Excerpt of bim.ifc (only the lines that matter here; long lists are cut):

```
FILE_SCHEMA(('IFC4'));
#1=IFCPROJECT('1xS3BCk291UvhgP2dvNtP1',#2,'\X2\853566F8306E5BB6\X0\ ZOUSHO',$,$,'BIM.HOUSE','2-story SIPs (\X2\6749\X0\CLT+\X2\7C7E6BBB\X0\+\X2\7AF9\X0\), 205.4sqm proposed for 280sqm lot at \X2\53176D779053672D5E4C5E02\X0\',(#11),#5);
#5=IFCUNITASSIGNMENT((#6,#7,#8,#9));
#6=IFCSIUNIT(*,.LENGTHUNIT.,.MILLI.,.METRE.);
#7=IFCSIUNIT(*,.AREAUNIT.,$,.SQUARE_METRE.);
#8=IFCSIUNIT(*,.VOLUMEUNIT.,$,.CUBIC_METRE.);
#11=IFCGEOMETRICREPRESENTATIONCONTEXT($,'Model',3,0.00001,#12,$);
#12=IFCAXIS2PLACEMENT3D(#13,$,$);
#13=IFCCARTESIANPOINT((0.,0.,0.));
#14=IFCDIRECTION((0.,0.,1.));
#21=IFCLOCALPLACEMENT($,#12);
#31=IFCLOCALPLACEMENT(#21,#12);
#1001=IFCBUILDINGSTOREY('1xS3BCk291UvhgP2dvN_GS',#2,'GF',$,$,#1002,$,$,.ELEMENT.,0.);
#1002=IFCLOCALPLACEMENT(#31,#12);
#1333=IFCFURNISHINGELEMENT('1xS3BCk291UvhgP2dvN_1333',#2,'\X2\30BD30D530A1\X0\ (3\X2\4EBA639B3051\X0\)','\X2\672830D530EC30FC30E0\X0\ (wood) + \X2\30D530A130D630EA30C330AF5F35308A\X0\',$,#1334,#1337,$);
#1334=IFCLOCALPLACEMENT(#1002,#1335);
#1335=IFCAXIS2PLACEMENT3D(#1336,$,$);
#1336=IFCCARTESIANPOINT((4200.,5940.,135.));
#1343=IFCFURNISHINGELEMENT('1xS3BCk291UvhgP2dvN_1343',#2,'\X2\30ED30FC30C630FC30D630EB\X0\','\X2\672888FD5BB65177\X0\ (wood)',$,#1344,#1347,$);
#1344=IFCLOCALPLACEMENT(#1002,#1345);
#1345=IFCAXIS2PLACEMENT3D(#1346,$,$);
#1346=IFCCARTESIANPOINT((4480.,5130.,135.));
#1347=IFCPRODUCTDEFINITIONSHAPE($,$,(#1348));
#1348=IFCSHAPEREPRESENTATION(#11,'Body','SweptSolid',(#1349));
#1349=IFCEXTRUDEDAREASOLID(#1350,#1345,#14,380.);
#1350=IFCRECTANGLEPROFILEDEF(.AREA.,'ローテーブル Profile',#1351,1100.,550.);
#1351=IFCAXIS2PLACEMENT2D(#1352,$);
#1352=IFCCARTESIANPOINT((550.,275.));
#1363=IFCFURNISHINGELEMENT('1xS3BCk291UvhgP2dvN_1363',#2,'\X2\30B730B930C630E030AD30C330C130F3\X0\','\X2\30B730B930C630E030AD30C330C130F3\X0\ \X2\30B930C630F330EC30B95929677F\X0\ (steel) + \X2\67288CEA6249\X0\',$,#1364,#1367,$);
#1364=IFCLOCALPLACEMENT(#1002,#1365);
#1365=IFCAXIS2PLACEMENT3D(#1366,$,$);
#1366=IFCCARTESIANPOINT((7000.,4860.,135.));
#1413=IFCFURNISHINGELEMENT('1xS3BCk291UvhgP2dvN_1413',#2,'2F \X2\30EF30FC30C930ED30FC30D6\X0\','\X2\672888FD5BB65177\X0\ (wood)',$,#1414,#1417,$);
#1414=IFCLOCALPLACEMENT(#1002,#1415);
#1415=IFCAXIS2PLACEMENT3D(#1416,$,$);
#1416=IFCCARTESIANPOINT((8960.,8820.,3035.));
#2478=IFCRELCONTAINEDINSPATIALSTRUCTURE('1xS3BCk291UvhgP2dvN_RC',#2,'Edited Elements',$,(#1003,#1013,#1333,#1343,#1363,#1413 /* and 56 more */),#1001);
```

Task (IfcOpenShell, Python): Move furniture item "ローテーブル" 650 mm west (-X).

```python
import ifcopenshell
import ifcopenshell.api.geometry
import ifcopenshell.util.placement
import ifcopenshell.util.unit

model = ifcopenshell.open("bim.ifc")
unit_scale = ifcopenshell.util.unit.calculate_unit_scale(model)

item = model.by_guid("1xS3BCk291UvhgP2dvN_1343")
matrix = ifcopenshell.util.placement.get_local_placement(item.ObjectPlacement)
matrix[0, 3] -= 0.65 / unit_scale
ifcopenshell.api.geometry.edit_object_placement(model, product=item, matrix=matrix, is_si=False)

print(ifcopenshell.util.placement.get_local_placement(item.ObjectPlacement).round(3) + 0.0)

model.write("bim_updated.ifc")
```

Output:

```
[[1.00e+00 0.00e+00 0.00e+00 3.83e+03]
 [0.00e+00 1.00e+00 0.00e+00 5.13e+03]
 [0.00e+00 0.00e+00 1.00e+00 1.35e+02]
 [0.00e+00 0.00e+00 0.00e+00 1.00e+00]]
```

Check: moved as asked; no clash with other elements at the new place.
